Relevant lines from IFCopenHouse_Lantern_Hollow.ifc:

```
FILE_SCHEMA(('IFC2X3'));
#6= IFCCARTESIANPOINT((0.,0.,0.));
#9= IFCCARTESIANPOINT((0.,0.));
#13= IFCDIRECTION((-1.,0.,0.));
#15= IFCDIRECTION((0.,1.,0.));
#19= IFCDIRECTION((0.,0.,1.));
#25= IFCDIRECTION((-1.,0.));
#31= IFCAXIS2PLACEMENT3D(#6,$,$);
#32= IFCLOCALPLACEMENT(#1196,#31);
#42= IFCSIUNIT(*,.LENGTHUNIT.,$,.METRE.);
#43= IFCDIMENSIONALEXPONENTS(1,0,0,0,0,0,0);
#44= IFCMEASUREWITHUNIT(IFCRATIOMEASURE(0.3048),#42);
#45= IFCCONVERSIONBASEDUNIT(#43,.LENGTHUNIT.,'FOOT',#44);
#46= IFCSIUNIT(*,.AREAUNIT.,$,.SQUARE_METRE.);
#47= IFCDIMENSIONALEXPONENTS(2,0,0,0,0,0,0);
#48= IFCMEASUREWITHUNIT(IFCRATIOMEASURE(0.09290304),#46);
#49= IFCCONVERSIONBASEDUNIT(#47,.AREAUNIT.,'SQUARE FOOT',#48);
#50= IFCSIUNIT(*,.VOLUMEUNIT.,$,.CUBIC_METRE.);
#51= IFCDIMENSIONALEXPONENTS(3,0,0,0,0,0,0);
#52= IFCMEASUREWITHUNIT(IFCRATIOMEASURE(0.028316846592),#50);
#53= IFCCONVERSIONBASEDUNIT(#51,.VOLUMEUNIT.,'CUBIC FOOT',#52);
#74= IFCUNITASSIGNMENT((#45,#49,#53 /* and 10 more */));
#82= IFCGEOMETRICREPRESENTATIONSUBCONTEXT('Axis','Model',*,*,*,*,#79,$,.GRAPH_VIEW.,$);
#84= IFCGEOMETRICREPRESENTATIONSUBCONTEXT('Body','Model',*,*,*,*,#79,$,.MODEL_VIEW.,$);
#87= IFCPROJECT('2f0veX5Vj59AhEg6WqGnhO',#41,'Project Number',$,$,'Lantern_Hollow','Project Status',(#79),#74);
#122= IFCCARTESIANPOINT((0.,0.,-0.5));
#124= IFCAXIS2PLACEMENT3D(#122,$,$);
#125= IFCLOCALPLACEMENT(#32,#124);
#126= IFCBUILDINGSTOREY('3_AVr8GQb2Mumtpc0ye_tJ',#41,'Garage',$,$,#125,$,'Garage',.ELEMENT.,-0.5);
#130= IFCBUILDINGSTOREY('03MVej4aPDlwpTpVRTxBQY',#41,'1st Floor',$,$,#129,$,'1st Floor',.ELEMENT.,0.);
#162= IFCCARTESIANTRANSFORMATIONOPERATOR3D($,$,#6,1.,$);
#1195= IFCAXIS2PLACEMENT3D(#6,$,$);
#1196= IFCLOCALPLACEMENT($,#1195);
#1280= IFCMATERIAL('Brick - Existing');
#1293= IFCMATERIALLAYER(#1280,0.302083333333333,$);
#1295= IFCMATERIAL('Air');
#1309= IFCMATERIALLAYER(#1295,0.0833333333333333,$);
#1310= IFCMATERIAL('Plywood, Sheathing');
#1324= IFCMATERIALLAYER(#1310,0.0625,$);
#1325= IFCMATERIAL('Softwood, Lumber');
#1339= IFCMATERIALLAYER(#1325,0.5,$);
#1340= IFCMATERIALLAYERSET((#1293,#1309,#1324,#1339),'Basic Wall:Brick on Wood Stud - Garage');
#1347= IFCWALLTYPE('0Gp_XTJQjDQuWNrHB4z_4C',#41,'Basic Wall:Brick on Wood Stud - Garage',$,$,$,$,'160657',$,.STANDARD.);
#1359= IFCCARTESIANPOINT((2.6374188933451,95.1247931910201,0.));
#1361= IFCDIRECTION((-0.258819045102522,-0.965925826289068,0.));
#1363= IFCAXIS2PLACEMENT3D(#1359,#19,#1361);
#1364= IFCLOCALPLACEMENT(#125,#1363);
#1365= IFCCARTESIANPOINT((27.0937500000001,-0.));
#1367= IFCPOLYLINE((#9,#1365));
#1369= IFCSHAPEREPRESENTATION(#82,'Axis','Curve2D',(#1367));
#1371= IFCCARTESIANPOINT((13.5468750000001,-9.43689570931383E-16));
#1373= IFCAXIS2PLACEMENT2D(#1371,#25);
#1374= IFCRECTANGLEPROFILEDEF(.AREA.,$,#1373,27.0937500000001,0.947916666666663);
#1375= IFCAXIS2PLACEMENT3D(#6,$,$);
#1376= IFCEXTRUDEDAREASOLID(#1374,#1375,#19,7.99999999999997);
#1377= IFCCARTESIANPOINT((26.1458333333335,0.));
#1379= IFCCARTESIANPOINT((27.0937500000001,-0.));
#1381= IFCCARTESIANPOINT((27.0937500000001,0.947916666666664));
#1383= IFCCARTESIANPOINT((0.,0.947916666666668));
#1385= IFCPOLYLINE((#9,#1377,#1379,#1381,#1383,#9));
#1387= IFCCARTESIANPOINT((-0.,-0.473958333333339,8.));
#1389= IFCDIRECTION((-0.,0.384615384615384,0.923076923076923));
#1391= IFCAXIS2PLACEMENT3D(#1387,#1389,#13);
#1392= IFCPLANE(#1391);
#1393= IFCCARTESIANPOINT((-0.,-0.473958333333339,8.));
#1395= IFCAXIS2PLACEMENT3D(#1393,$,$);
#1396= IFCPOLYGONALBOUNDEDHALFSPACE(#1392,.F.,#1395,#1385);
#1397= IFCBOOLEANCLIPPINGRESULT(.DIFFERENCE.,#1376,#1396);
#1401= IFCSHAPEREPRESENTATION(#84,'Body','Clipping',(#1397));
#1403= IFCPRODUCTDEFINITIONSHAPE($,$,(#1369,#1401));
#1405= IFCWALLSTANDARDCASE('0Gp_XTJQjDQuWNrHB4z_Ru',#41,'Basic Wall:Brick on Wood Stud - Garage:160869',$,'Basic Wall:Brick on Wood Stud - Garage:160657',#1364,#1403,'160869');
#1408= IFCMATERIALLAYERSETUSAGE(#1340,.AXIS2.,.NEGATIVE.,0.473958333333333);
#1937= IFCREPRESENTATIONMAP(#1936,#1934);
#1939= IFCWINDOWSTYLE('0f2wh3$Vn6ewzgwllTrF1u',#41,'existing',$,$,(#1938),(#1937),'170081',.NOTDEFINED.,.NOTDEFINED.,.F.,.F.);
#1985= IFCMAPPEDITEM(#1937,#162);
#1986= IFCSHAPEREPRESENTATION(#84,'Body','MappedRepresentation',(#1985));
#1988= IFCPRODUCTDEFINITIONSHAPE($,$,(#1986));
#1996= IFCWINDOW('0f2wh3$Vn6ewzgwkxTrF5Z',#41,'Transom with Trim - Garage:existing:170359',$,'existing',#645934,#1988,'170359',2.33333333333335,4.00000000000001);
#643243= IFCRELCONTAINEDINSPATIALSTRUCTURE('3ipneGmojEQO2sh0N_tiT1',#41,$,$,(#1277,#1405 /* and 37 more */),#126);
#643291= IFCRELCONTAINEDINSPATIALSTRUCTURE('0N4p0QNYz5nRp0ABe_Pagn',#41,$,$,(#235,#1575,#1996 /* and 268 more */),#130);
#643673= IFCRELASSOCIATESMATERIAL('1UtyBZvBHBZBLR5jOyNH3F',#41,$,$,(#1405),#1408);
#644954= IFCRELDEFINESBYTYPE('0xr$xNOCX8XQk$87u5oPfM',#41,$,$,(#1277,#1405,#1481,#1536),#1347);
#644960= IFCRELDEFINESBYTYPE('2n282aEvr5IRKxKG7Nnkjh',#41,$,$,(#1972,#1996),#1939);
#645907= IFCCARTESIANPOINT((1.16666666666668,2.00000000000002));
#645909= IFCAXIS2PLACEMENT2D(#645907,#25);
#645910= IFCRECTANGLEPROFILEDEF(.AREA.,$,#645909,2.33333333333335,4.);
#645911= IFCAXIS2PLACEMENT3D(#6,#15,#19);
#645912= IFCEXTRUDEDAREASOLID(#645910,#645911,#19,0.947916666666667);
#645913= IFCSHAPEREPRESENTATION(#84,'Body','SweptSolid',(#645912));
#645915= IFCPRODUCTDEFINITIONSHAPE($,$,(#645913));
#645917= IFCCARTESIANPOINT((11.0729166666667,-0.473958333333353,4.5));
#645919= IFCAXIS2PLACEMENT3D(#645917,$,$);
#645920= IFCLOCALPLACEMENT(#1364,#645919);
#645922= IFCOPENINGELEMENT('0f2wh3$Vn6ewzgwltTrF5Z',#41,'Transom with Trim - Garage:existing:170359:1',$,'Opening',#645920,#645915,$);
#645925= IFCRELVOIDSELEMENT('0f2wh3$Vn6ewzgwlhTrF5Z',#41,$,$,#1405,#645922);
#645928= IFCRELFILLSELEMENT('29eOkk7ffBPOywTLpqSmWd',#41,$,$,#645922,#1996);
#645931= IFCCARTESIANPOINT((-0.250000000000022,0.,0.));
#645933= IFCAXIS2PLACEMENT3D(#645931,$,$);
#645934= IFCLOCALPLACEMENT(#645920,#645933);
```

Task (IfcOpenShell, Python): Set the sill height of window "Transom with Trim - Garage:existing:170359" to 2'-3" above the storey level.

```python
import numpy as np
import ifcopenshell
import ifcopenshell.api.geometry
import ifcopenshell.geom
import ifcopenshell.util.element
import ifcopenshell.util.placement
import ifcopenshell.util.shape
import ifcopenshell.util.unit

model = ifcopenshell.open("IFCopenHouse_Lantern_Hollow.ifc")
unit_scale = ifcopenshell.util.unit.calculate_unit_scale(model)

window = model.by_id(1996)
opening = window.FillsVoids[0].RelatingOpeningElement
storey = ifcopenshell.util.element.get_container(window, ifc_class="IfcBuildingStorey")
level = ifcopenshell.util.placement.get_local_placement(storey.ObjectPlacement)[2, 3]

# The opening's origin need not be at the sill, so measure its lowest point.
shape = ifcopenshell.geom.create_shape(ifcopenshell.geom.settings(), opening)
bottom = ifcopenshell.util.shape.get_shape_bottom_elevation(shape, shape.geometry) / unit_scale
dz = level + 27 * 0.0254 / unit_scale - bottom

shift = np.array([0.0, 0.0, dz])
# The window is placed relative to its opening, so it follows when the opening moves.
matrix = ifcopenshell.util.placement.get_local_placement(opening.ObjectPlacement)
matrix[:3, 3] += shift
ifcopenshell.api.geometry.edit_object_placement(
    model, product=opening, matrix=matrix, is_si=False, should_transform_children=True
)

print(f"moved by {dz * unit_scale:+.3f} m")

model.write("IFCopenHouse_Lantern_Hollow_edited.ifc")
```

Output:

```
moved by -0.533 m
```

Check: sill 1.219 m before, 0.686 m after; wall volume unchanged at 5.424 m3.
